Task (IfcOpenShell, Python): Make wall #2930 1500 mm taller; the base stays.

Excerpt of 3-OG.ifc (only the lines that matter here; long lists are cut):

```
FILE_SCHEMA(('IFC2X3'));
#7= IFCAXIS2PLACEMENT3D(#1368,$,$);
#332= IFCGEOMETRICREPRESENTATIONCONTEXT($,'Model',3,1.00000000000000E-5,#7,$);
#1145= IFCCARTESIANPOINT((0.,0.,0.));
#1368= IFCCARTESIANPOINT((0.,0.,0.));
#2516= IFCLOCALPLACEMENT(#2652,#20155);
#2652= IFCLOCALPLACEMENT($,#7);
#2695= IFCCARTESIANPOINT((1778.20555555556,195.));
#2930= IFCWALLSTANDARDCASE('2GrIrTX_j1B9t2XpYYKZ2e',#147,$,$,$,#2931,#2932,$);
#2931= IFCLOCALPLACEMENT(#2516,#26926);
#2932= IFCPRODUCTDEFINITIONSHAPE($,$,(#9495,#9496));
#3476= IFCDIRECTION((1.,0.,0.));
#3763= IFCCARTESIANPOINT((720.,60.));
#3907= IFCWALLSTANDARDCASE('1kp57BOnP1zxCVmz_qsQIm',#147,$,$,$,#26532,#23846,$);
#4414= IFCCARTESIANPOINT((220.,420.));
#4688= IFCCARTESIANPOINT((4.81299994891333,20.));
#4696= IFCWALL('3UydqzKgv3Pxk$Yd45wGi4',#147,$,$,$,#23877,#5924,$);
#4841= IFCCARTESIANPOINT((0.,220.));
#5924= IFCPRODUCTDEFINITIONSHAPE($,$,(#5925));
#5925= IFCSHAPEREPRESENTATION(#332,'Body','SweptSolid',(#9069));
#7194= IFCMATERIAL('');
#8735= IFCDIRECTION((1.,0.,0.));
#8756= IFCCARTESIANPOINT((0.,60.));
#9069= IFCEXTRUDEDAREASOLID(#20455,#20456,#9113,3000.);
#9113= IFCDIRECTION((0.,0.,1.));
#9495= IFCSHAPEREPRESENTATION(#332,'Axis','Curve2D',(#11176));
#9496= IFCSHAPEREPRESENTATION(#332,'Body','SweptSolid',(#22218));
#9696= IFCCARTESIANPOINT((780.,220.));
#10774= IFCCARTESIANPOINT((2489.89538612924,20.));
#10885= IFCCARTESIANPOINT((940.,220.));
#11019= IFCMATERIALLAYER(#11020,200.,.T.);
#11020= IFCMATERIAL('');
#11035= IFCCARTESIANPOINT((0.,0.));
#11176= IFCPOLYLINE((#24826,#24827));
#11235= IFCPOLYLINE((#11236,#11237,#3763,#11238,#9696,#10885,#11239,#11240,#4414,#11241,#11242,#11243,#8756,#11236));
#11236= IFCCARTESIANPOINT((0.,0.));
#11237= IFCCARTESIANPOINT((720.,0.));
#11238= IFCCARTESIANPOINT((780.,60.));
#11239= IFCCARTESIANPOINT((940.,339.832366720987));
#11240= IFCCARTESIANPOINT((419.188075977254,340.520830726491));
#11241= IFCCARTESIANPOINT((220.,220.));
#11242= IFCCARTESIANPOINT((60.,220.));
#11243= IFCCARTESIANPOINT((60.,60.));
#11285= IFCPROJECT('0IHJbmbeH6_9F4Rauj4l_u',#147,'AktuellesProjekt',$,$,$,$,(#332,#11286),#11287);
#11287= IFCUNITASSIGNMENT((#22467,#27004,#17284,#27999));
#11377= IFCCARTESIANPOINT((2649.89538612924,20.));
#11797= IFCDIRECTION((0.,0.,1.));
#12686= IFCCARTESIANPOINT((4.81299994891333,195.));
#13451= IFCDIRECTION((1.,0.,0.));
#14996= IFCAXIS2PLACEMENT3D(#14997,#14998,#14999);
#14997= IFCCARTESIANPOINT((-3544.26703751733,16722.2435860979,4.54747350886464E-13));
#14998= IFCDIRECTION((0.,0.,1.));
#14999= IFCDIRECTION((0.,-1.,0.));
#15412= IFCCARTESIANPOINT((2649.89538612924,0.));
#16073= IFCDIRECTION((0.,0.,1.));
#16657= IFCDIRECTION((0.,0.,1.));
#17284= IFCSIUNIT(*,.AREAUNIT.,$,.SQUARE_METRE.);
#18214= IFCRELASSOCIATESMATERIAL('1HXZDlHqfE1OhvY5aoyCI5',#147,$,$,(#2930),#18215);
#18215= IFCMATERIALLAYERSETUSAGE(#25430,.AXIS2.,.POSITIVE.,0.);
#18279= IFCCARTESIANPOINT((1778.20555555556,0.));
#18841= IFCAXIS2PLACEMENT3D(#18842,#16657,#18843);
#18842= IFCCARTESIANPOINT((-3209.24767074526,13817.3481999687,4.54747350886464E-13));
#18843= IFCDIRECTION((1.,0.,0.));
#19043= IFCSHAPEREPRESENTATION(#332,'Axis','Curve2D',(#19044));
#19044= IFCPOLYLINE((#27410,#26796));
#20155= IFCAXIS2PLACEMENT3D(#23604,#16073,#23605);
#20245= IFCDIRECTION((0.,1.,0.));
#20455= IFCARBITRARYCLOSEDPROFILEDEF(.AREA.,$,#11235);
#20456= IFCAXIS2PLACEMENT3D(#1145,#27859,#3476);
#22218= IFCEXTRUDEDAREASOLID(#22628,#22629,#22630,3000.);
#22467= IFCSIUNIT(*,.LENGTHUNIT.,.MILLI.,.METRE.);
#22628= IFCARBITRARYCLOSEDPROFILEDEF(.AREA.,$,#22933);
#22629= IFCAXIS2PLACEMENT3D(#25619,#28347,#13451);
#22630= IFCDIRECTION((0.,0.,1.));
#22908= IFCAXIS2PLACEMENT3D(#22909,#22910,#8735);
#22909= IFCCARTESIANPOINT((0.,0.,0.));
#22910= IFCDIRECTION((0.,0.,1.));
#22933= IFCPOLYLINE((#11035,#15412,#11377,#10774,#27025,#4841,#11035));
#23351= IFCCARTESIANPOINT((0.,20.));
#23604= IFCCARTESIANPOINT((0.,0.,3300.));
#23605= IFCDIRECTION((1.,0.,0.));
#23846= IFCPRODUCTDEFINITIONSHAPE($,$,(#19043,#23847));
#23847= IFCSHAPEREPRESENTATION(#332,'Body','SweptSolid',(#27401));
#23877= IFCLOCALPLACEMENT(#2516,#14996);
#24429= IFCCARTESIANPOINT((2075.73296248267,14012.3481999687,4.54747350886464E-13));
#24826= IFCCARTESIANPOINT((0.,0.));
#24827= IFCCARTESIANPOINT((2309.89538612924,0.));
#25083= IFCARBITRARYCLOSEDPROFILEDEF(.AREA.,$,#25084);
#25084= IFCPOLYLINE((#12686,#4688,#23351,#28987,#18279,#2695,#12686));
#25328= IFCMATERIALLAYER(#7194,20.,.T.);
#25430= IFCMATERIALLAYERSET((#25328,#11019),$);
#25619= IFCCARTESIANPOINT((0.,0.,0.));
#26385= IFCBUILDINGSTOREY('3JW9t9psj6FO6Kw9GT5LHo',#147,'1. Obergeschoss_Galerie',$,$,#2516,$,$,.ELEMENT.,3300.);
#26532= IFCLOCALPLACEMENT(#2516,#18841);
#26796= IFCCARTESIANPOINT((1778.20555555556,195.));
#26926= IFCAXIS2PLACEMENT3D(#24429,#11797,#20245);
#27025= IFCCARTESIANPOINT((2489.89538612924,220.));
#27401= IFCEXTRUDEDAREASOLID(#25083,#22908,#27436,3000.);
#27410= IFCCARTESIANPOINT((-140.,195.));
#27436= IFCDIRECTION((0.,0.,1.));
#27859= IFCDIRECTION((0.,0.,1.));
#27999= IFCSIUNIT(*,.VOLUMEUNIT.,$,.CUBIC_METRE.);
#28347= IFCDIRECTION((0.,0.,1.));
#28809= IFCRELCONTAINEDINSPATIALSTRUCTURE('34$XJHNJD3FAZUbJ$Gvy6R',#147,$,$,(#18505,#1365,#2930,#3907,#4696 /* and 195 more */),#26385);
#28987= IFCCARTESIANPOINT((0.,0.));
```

```python
import ifcopenshell
import ifcopenshell.geom
import ifcopenshell.util.shape
import ifcopenshell.util.unit

model = ifcopenshell.open("3-OG.ifc")
unit_scale = ifcopenshell.util.unit.calculate_unit_scale(model)
settings = ifcopenshell.geom.settings()


def volume(element):
    """Net volume in cubic metres, openings subtracted."""
    shape = ifcopenshell.geom.create_shape(settings, element)
    return ifcopenshell.util.shape.get_volume(shape.geometry)


wall = model.by_guid("2GrIrTX_j1B9t2XpYYKZ2e")
before = volume(wall)

body = next(r for r in wall.Representation.Representations if r.RepresentationIdentifier == "Body")
solid = body.Items[0]
old_height = solid.Depth
solid.Depth += 1.5 / unit_scale
after = volume(wall)

print(f"height {old_height:g} -> {solid.Depth:g}, volume {before:.3f} -> {after:.3f} m3")

model.write("3-OG-out.ifc")
```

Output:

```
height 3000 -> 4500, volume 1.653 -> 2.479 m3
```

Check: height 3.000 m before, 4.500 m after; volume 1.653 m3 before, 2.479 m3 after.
